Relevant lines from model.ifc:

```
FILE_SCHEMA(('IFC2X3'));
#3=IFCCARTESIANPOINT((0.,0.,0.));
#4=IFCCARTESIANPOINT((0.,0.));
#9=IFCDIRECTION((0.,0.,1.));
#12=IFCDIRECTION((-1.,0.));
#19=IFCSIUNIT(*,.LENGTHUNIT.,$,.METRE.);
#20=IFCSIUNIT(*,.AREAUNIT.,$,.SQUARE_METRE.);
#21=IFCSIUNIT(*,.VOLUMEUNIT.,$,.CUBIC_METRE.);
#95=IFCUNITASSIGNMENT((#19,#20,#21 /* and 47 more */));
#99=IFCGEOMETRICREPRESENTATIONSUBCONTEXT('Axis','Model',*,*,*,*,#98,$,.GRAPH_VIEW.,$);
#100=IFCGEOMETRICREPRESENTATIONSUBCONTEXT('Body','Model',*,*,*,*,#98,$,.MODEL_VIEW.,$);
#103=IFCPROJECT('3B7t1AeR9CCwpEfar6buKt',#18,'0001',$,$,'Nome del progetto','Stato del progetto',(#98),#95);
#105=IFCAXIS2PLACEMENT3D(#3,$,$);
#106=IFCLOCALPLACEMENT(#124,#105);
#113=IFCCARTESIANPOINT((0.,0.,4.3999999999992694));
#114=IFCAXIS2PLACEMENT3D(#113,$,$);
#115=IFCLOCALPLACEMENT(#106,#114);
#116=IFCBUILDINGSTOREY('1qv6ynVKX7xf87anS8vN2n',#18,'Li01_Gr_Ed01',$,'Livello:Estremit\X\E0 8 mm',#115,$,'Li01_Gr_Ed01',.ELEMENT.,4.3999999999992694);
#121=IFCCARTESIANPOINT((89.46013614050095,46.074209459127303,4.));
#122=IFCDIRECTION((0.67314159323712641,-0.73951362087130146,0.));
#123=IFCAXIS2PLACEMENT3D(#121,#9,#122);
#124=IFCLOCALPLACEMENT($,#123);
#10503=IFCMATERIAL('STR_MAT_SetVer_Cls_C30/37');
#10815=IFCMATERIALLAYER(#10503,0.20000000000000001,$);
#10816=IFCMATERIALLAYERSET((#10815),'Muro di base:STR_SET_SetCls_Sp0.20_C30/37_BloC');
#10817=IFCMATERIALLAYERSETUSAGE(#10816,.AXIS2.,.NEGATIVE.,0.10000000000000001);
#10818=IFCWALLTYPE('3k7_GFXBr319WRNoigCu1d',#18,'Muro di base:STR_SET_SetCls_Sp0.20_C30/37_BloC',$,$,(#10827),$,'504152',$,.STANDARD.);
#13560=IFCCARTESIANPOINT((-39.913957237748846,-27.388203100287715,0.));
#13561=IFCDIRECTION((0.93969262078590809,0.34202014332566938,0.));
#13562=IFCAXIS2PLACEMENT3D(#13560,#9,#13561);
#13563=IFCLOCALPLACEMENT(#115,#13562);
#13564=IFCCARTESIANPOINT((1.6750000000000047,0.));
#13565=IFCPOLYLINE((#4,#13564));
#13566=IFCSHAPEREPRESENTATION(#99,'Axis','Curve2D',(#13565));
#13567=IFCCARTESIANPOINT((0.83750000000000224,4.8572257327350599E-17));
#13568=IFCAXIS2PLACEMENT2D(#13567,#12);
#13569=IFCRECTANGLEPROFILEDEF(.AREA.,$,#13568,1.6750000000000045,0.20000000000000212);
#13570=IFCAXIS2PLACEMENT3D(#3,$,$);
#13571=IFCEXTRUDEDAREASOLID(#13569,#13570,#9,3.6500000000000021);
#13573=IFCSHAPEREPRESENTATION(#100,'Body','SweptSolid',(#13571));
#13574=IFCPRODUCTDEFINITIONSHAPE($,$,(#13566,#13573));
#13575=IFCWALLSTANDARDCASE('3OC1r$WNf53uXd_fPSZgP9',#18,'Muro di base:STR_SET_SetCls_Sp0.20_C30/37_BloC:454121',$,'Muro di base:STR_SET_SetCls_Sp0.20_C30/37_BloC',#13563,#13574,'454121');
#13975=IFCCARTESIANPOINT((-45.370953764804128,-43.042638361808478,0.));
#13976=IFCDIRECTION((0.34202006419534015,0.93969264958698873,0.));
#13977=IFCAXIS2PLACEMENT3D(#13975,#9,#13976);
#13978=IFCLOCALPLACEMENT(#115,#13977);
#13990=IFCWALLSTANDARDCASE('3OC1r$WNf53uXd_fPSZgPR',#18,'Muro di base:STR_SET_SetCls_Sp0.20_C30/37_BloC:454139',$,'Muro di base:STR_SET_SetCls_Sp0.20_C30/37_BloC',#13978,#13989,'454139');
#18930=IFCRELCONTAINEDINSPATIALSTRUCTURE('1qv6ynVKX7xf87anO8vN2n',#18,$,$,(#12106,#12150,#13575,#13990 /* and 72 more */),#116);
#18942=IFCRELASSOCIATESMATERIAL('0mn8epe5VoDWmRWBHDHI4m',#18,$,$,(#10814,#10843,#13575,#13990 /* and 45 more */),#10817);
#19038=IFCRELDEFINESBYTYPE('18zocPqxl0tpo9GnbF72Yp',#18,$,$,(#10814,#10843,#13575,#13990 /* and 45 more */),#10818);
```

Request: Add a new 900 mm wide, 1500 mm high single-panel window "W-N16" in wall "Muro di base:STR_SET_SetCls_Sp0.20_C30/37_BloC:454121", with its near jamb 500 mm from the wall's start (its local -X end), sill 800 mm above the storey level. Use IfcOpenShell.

```python
import numpy as np
import ifcopenshell
import ifcopenshell.api.feature
import ifcopenshell.api.geometry
import ifcopenshell.api.root
import ifcopenshell.api.spatial
import ifcopenshell.api.type
import ifcopenshell.geom
import ifcopenshell.util.element
import ifcopenshell.util.placement
import ifcopenshell.util.representation
import ifcopenshell.util.shape
import ifcopenshell.util.unit

model = ifcopenshell.open("model.ifc")
unit_scale = ifcopenshell.util.unit.calculate_unit_scale(model)
settings = ifcopenshell.geom.settings()


def volume(element):
    """Net volume in cubic metres, openings subtracted."""
    shape = ifcopenshell.geom.create_shape(settings, element)
    return ifcopenshell.util.shape.get_volume(shape.geometry)


wall = model.by_guid("3OC1r$WNf53uXd_fPSZgP9")
storey = ifcopenshell.util.element.get_container(wall, ifc_class="IfcBuildingStorey")
context = ifcopenshell.util.representation.get_context(model, "Model", "Body", "MODEL_VIEW")
before = volume(wall)

width, height, from_end, sill = 0.9, 1.5, 0.5, 0.8  # metres

# The wall runs along its own X axis, and the end named is its -X end.
wall_shape = ifcopenshell.geom.create_shape(settings, wall)
x, y, z = ifcopenshell.util.shape.get_vertices(wall_shape.geometry).T
start = x.min() + from_end
face, thickness = float(y.min()), float(y.max() - y.min())
wall_matrix = ifcopenshell.util.placement.get_local_placement(wall.ObjectPlacement)
level = ifcopenshell.util.placement.get_local_placement(storey.ObjectPlacement)[2, 3]


def in_wall(x, y):
    """Placement at x, y metres in the wall's axes, at sill height."""
    matrix = wall_matrix.copy()
    matrix[:, 3] = wall_matrix @ np.array([x / unit_scale, y / unit_scale, 0.0, 1.0])
    matrix[2, 3] = level + sill / unit_scale
    return matrix


# Opening: a box that overshoots both wall faces by 50 mm.
opening = ifcopenshell.api.root.create_entity(model, ifc_class="IfcOpeningElement")
box = ifcopenshell.api.geometry.add_wall_representation(
    model, context=context, length=width, height=height, thickness=thickness + 0.1
)
ifcopenshell.api.geometry.assign_representation(model, product=opening, representation=box)
ifcopenshell.api.geometry.edit_object_placement(model, product=opening, matrix=in_wall(start, face - 0.05), is_si=False)
ifcopenshell.api.feature.add_feature(model, feature=opening, element=wall)

window = ifcopenshell.api.root.create_entity(model, ifc_class="IfcWindow", name="W-N16")
window.OverallWidth, window.OverallHeight = width / unit_scale, height / unit_scale
body = ifcopenshell.api.geometry.add_window_representation(
    model,
    context=context,
    overall_width=window.OverallWidth,
    overall_height=window.OverallHeight,
    partition_type="SINGLE_PANEL",
)
ifcopenshell.api.geometry.assign_representation(model, product=window, representation=body)
ifcopenshell.api.spatial.assign_container(model, products=[window], relating_structure=storey)
fills = ifcopenshell.api.feature.add_filling(model, opening=opening, element=window)
fills.OwnerHistory = window.OwnerHistory  # required in IFC2X3

# IFC2X3 keeps the operation on the window style.
style = ifcopenshell.api.root.create_entity(model, ifc_class="IfcWindowStyle", name="W-N16")
style.OperationType, style.ConstructionType = "SINGLE_PANEL", "NOTDEFINED"
style.ParameterTakesPrecedence = style.Sizeable = False
ifcopenshell.api.type.assign_type(model, related_objects=[window], relating_type=style)

# Centre the window in the wall's thickness.
ifcopenshell.api.geometry.edit_object_placement(model, product=window, matrix=in_wall(start, face), is_si=False)
window_shape = ifcopenshell.geom.create_shape(settings, window)
depth = ifcopenshell.util.shape.get_vertices(window_shape.geometry)[:, 1]
offset = face + thickness / 2 - (depth.min() + depth.max()) / 2
ifcopenshell.api.geometry.edit_object_placement(model, product=window, matrix=in_wall(start, offset), is_si=False)

after = volume(wall)

print(f"wall volume {before:.3f} -> {after:.3f} m3")

model.write("model_v2.ifc")
```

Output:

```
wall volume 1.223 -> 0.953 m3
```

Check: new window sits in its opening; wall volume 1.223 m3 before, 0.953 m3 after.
